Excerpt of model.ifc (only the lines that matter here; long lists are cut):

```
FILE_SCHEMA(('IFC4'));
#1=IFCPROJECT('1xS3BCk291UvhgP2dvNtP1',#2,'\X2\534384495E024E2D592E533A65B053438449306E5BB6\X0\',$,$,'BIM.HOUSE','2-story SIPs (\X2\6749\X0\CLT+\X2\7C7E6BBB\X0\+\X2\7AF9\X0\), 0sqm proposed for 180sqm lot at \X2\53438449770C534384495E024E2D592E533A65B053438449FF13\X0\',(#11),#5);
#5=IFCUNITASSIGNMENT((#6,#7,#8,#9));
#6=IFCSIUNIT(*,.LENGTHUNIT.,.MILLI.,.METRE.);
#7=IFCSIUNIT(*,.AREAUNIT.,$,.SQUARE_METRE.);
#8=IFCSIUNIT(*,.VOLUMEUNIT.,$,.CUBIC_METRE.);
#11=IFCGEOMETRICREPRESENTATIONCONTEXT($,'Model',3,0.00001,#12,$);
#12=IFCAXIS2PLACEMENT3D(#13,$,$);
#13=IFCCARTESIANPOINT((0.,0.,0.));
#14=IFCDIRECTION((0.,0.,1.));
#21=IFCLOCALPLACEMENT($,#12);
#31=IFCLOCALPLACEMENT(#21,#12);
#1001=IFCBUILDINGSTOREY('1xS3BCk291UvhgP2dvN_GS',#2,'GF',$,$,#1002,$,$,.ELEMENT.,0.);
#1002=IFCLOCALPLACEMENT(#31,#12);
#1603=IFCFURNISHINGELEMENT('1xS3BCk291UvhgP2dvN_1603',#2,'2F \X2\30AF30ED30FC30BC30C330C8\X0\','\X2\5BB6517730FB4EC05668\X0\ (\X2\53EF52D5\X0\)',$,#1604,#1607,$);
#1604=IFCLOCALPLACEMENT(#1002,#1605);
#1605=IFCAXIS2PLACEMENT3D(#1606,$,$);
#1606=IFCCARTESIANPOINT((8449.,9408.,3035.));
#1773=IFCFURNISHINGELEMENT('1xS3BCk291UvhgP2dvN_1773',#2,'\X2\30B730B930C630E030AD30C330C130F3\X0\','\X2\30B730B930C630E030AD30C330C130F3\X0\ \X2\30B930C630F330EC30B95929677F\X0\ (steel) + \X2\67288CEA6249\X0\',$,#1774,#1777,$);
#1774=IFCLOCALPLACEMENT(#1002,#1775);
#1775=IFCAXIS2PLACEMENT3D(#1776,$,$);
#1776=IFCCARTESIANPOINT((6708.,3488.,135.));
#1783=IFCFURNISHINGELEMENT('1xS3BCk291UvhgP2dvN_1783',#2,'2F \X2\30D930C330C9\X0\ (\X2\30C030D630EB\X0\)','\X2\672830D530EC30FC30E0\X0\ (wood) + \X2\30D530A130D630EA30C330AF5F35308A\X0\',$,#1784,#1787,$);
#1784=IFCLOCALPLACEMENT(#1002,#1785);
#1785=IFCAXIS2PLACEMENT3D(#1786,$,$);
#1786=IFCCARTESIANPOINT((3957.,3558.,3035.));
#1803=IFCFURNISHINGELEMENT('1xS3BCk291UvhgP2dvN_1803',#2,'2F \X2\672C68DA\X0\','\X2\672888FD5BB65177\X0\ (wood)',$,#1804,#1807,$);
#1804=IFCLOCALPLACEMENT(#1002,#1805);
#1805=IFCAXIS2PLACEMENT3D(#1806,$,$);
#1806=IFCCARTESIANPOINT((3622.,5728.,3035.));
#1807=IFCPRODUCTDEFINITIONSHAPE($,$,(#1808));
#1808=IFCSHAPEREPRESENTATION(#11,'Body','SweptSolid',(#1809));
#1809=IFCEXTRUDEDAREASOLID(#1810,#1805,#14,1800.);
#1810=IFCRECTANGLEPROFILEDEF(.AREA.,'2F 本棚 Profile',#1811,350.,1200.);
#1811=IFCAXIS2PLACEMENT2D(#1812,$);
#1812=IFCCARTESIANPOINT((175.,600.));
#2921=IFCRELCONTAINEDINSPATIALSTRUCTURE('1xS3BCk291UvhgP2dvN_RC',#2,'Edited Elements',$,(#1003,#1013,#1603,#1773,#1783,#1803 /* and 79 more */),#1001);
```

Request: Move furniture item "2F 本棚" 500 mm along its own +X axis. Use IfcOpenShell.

```python
import ifcopenshell
import ifcopenshell.api.geometry
import ifcopenshell.util.placement

model = ifcopenshell.open("model.ifc")

item = model.by_guid("1xS3BCk291UvhgP2dvN_1803")
matrix = ifcopenshell.util.placement.get_local_placement(item.ObjectPlacement)
matrix[:3, 3] += matrix[:3, 0] * 500.0
ifcopenshell.api.geometry.edit_object_placement(model, product=item, matrix=matrix, is_si=False)

print(ifcopenshell.util.placement.get_local_placement(item.ObjectPlacement).round(3) + 0.0)

model.write("model_updated.ifc")
```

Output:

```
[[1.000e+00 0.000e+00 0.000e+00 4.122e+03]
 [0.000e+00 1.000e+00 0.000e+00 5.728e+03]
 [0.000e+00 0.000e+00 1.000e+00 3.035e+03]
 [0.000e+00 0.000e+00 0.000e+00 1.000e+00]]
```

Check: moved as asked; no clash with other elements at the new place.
